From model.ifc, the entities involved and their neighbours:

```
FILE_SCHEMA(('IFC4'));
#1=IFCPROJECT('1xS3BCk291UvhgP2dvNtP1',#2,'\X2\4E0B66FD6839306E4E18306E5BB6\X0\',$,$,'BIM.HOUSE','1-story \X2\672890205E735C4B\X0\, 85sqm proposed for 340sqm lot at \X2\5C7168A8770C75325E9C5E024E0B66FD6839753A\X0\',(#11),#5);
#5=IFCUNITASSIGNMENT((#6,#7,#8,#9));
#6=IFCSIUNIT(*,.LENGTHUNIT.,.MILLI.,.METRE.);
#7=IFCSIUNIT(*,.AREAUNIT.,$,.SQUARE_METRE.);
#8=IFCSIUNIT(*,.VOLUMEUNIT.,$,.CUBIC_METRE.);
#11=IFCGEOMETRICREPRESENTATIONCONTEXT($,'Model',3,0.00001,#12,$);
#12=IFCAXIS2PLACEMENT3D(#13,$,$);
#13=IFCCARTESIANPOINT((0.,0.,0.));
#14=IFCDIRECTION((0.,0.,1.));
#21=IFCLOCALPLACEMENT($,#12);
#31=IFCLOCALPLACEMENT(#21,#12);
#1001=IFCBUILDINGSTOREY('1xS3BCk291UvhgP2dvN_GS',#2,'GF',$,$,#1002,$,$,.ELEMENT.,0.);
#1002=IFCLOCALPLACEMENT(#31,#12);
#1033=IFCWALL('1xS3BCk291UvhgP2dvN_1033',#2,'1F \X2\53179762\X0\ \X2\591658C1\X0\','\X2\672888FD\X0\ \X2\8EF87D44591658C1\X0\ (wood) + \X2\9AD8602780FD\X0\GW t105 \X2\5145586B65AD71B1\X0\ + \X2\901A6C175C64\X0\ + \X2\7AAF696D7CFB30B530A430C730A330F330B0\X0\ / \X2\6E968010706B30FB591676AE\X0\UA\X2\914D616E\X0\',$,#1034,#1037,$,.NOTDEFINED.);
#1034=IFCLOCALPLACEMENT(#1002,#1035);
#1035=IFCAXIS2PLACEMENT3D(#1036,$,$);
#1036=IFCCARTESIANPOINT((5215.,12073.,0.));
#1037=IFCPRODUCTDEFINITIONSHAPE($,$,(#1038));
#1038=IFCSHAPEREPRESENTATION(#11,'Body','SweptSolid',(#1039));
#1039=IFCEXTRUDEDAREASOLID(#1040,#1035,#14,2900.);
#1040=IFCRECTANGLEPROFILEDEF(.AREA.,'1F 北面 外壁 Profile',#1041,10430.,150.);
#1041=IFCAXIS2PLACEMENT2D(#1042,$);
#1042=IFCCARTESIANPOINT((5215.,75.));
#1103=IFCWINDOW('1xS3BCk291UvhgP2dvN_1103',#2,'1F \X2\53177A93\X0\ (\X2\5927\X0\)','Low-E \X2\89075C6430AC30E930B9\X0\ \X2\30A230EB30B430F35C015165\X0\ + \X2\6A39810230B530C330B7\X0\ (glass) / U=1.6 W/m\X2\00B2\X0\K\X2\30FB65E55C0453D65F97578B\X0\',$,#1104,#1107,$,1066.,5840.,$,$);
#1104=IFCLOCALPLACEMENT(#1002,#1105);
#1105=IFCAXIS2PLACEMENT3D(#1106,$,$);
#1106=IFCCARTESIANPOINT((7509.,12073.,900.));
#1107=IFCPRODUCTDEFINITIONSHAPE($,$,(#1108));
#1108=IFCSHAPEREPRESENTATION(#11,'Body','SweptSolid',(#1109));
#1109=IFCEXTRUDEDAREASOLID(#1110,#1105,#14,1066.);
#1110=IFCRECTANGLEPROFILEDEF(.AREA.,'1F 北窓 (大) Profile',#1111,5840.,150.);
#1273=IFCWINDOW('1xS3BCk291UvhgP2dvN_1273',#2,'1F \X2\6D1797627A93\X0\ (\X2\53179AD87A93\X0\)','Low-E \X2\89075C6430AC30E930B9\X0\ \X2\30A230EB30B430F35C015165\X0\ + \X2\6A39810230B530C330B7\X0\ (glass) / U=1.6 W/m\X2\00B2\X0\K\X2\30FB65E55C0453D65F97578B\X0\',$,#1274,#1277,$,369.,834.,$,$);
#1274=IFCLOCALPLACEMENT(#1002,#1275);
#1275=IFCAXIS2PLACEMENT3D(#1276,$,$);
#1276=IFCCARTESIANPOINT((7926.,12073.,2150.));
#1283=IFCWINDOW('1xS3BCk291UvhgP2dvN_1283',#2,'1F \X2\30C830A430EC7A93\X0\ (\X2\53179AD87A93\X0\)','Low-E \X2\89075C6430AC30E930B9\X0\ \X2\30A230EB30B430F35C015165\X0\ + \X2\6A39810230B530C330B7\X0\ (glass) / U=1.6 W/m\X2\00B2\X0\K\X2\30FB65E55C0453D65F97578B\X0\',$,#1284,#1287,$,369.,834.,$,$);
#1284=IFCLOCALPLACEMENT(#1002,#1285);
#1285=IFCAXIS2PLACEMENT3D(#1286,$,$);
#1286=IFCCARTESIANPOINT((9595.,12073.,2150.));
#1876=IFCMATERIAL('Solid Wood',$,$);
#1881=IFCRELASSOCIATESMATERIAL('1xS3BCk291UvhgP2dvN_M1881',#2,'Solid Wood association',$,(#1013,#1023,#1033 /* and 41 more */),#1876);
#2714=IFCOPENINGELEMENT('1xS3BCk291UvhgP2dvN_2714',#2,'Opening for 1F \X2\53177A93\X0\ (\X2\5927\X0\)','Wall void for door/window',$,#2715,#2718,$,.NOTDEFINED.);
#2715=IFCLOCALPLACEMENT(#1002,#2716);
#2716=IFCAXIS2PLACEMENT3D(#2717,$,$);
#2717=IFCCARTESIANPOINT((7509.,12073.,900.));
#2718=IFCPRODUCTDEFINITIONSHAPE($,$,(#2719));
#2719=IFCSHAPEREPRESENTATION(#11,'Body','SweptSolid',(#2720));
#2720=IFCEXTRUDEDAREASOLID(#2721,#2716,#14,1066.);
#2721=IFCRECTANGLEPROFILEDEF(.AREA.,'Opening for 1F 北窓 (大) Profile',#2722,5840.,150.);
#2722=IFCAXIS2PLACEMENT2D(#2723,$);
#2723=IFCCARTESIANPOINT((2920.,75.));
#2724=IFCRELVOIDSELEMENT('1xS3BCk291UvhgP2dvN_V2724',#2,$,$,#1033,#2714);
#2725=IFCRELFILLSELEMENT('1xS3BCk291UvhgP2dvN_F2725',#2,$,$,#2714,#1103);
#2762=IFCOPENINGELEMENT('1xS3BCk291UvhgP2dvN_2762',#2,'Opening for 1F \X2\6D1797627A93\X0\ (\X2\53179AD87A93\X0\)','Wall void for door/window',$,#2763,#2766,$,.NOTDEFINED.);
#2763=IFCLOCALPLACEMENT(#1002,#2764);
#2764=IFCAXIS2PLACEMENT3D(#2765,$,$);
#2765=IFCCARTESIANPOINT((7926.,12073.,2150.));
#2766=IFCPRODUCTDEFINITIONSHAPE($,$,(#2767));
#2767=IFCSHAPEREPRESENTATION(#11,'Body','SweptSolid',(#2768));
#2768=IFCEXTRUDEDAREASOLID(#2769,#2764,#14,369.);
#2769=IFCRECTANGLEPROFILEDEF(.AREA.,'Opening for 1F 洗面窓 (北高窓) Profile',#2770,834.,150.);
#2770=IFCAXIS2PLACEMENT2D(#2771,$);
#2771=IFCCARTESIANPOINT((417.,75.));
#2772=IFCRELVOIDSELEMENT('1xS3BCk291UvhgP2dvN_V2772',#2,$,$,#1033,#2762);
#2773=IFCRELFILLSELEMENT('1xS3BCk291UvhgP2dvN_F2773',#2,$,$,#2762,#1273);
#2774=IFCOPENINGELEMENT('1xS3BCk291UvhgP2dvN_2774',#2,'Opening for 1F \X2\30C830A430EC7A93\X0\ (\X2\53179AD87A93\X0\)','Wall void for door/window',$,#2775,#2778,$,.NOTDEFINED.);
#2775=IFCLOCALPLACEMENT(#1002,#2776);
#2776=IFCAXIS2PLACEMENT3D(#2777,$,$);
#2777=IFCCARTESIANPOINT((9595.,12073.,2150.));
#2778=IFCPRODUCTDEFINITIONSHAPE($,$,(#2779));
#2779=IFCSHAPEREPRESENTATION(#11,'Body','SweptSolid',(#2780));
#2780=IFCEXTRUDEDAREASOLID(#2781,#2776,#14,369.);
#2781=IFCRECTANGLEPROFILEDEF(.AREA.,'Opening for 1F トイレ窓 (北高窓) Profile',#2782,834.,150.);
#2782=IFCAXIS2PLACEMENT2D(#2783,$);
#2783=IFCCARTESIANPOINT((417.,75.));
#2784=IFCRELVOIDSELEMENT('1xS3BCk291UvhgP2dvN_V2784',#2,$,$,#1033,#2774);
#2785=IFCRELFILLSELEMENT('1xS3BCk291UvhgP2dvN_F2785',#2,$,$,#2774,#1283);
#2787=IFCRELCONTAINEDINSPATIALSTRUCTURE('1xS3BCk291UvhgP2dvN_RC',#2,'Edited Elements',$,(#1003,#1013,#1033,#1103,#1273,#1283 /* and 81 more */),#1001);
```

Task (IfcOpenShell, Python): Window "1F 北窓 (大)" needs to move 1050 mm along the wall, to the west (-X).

```python
import ifcopenshell
import ifcopenshell.api.geometry
import ifcopenshell.util.placement

model = ifcopenshell.open("model.ifc")

window = model.by_guid("1xS3BCk291UvhgP2dvN_1103")
opening = window.FillsVoids[0].RelatingOpeningElement
wall = opening.VoidsElements[0].RelatingBuildingElement

wall_matrix = ifcopenshell.util.placement.get_local_placement(wall.ObjectPlacement)
shift = wall_matrix[:3, 0] * -1050.0
before = ifcopenshell.util.placement.get_local_placement(window.ObjectPlacement)[:3, 3].copy()

# The window is not placed relative to its opening, so move both.
for product in (opening, window):
    matrix = ifcopenshell.util.placement.get_local_placement(product.ObjectPlacement)
    matrix[:3, 3] += shift
    ifcopenshell.api.geometry.edit_object_placement(model, product=product, matrix=matrix, is_si=False)

after = ifcopenshell.util.placement.get_local_placement(window.ObjectPlacement)[:3, 3]
print("window moved by", (after - before).round(3) + 0.0)

model.write("model_edited.ifc")
```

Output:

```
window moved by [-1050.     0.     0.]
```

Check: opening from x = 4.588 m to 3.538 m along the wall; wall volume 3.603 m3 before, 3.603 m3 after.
